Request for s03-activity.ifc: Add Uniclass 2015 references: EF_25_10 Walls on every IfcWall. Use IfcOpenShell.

First a look at what the model holds.

```python
import ifcopenshell

model = ifcopenshell.open("s03-activity.ifc")
print(model.schema)
print("classifications:", [c.Name for c in model.by_type("IfcClassification")])
for ifc_class in ("IfcDoor", "IfcRoof", "IfcStair", "IfcWall", "IfcWindow"):
    print(ifc_class, len(model.by_type(ifc_class)))
```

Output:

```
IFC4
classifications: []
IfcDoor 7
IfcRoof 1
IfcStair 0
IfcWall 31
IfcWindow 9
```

```python
import ifcopenshell
import ifcopenshell.api.classification

model = ifcopenshell.open("s03-activity.ifc")

system = ifcopenshell.api.classification.add_classification(model, classification="Uniclass 2015")

codes = {
    "IfcWall": ("EF_25_10", "Walls"),
}
for ifc_class, (code, name) in codes.items():
    products = model.by_type(ifc_class)
    ifcopenshell.api.classification.add_reference(
        model, products=products, classification=system, identification=code, name=name
    )
    print(code, len(products))

model.write("s03-activity_updated.ifc")
```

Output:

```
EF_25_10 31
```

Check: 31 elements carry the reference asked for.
